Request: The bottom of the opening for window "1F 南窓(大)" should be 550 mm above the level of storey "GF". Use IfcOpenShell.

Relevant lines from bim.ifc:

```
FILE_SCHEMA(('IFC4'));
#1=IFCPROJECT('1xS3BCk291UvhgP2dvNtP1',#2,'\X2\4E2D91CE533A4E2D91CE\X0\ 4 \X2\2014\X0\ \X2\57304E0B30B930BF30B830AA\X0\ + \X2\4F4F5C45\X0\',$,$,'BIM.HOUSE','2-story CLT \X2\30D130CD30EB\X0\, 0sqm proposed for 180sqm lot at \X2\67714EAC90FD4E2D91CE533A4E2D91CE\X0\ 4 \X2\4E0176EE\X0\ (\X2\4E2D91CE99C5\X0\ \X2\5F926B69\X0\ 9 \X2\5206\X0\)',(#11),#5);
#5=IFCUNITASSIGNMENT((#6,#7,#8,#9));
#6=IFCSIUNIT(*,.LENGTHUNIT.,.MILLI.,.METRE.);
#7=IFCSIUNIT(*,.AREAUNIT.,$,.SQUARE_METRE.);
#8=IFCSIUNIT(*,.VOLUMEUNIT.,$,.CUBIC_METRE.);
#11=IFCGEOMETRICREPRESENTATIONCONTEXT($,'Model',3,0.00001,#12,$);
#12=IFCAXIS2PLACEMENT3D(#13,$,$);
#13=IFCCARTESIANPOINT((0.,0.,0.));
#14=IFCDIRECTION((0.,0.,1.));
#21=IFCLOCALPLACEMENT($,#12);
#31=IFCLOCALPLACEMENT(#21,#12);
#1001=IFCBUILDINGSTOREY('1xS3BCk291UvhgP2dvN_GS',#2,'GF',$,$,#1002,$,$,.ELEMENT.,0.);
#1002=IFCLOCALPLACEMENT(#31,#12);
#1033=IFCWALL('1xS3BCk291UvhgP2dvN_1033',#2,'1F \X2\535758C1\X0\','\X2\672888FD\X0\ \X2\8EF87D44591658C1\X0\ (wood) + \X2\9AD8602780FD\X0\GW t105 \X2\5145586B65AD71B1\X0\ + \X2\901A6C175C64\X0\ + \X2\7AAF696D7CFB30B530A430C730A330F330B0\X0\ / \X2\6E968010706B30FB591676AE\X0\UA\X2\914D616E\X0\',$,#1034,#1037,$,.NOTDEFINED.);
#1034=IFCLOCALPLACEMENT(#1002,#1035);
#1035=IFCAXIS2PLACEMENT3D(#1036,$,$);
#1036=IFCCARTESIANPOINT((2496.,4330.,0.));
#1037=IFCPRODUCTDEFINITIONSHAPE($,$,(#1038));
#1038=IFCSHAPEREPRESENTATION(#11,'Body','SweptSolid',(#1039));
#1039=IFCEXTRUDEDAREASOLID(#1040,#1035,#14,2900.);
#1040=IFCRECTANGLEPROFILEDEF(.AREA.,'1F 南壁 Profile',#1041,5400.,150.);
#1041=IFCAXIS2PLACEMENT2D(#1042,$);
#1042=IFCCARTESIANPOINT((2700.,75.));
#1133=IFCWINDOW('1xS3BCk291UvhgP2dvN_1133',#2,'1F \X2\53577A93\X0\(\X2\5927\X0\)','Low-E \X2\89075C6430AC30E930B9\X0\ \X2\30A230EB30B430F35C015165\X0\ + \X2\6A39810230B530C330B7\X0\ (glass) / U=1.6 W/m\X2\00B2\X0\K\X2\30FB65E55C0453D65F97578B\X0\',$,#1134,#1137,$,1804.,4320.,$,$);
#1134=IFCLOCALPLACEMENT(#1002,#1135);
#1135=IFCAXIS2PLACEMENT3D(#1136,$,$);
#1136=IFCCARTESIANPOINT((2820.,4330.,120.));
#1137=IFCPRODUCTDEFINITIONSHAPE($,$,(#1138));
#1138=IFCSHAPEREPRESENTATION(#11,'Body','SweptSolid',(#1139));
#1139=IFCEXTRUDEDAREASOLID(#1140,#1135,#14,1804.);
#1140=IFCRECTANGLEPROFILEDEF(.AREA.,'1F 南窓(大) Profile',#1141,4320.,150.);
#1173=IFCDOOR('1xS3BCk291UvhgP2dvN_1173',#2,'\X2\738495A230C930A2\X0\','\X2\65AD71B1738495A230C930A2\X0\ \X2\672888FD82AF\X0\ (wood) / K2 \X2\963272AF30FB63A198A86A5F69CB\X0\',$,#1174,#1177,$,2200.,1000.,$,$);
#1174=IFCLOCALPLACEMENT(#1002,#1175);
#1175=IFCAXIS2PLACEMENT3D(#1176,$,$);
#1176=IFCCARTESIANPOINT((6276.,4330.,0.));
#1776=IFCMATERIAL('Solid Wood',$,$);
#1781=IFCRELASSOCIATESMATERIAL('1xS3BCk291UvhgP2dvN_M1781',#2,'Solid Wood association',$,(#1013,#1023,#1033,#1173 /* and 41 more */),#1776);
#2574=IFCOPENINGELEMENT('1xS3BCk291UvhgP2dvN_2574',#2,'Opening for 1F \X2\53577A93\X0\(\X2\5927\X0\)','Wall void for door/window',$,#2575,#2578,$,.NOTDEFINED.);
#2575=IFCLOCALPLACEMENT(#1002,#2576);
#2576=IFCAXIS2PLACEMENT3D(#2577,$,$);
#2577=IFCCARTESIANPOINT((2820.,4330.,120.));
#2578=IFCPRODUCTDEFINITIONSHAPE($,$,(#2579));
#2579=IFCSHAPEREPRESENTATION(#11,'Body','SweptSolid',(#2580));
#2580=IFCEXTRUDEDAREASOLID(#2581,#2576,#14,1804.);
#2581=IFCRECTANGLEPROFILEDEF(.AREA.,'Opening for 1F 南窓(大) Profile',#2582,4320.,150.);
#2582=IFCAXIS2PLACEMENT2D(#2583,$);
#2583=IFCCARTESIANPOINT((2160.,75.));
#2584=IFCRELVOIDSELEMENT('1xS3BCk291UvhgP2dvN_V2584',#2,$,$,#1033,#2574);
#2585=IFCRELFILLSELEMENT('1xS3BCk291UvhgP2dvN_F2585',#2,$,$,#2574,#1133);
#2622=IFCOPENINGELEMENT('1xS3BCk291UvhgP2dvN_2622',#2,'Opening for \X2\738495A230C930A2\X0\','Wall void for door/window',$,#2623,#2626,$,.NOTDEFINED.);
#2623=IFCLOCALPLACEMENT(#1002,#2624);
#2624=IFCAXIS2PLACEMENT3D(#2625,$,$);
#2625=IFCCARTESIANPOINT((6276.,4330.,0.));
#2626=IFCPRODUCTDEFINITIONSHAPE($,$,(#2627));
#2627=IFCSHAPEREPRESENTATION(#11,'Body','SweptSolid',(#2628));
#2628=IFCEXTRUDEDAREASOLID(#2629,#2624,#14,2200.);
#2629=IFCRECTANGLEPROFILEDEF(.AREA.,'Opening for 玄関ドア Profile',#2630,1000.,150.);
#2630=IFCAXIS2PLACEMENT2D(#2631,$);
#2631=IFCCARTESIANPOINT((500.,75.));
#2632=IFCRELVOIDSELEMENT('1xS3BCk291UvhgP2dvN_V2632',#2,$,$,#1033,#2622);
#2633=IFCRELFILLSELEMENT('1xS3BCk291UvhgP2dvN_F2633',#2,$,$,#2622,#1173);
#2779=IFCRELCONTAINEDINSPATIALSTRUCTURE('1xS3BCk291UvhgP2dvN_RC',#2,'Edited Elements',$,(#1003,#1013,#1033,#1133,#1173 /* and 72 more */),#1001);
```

```python
import numpy as np
import ifcopenshell
import ifcopenshell.api.geometry
import ifcopenshell.geom
import ifcopenshell.util.element
import ifcopenshell.util.placement
import ifcopenshell.util.shape
import ifcopenshell.util.unit

model = ifcopenshell.open("bim.ifc")
unit_scale = ifcopenshell.util.unit.calculate_unit_scale(model)

window = model.by_id(1133)
opening = window.FillsVoids[0].RelatingOpeningElement
storey = ifcopenshell.util.element.get_container(window, ifc_class="IfcBuildingStorey")
level = ifcopenshell.util.placement.get_local_placement(storey.ObjectPlacement)[2, 3]

# The opening's origin need not be at the sill, so measure its lowest point.
shape = ifcopenshell.geom.create_shape(ifcopenshell.geom.settings(), opening)
bottom = ifcopenshell.util.shape.get_shape_bottom_elevation(shape, shape.geometry) / unit_scale
dz = level + 550.0 - bottom

shift = np.array([0.0, 0.0, dz])
# The window is not placed relative to its opening, so move both.
for product in (opening, window):
    matrix = ifcopenshell.util.placement.get_local_placement(product.ObjectPlacement)
    matrix[:3, 3] += shift
    ifcopenshell.api.geometry.edit_object_placement(model, product=product, matrix=matrix, is_si=False)

print(f"moved by {dz * unit_scale:+.3f} m")

model.write("bim-out.ifc")
```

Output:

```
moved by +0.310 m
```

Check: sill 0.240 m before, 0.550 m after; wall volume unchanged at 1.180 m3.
